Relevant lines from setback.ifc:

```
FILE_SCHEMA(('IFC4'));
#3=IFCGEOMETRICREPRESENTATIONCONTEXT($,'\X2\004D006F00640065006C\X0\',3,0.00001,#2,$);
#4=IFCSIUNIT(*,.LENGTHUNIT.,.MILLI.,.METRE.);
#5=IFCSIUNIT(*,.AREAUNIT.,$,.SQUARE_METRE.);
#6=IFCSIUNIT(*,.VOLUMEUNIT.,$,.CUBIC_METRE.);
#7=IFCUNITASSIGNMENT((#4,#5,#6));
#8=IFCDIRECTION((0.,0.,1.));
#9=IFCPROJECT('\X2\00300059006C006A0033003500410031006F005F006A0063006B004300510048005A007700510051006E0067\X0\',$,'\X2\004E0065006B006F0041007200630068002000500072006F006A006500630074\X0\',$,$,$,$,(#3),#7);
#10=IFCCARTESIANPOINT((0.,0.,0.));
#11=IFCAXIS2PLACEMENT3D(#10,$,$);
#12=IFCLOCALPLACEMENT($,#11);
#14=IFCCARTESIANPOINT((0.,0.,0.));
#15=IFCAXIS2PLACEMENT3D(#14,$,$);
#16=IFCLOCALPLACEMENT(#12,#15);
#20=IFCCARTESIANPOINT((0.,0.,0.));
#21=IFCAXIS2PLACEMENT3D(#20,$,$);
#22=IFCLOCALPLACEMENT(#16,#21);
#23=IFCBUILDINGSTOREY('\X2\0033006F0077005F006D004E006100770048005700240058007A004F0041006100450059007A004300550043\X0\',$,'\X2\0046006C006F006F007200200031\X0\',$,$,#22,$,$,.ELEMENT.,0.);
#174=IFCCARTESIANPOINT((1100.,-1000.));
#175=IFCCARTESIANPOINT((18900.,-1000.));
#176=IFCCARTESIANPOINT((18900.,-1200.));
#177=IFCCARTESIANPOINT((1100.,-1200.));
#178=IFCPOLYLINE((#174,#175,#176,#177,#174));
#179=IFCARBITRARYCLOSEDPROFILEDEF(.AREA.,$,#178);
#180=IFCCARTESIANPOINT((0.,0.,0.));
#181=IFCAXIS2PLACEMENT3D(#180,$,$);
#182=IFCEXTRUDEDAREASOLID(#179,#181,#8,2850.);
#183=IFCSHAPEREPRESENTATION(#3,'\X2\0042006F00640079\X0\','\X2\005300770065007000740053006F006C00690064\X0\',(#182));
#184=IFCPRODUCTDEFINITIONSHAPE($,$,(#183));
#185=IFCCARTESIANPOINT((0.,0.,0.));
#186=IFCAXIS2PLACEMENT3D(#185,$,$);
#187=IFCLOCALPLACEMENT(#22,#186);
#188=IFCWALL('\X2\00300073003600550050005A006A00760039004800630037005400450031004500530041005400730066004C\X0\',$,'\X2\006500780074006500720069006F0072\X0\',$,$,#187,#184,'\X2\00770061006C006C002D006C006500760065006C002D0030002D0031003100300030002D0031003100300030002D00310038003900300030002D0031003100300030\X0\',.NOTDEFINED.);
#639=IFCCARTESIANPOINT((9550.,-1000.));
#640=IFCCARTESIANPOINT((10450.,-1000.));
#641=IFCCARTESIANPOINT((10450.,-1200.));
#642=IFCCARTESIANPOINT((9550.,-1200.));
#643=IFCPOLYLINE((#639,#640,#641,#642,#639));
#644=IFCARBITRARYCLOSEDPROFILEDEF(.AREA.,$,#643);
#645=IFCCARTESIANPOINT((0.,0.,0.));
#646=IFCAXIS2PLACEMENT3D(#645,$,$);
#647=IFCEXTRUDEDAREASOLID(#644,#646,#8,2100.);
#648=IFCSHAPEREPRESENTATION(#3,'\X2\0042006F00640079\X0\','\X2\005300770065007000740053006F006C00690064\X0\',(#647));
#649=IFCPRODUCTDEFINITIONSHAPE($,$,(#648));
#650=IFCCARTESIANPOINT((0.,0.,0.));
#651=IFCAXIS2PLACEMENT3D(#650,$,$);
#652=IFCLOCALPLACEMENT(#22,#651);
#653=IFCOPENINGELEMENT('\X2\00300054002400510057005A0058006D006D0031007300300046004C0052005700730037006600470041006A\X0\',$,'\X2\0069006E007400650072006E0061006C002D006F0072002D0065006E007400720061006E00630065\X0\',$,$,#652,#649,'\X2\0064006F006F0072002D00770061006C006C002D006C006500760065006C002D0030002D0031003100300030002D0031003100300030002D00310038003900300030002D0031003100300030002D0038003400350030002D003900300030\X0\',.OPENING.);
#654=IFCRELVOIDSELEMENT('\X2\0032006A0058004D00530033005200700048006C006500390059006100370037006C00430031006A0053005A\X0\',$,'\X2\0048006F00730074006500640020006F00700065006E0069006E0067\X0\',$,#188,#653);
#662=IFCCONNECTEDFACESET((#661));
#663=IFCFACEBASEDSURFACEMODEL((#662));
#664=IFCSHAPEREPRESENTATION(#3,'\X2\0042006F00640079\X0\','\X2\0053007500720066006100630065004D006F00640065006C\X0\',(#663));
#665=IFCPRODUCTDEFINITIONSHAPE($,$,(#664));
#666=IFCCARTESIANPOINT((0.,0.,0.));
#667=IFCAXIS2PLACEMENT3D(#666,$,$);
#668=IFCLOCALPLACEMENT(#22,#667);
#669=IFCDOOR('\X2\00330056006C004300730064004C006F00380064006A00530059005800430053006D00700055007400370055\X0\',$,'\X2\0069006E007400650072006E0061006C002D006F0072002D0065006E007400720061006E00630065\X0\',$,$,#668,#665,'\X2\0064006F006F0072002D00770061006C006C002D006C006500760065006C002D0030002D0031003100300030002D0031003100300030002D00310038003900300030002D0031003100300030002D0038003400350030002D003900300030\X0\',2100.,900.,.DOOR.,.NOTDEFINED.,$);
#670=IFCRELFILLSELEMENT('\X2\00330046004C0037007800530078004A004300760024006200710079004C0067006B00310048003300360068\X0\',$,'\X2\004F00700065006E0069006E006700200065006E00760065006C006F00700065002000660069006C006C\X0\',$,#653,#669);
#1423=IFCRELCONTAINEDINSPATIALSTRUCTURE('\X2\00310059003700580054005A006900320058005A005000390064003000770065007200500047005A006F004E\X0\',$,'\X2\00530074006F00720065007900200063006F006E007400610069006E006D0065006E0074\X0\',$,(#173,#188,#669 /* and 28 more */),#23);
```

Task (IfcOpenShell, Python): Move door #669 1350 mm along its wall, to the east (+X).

```python
import ifcopenshell
import ifcopenshell.api.geometry
import ifcopenshell.util.placement
import ifcopenshell.util.unit

model = ifcopenshell.open("setback.ifc")
unit_scale = ifcopenshell.util.unit.calculate_unit_scale(model)

door = model.by_id(669)
opening = door.FillsVoids[0].RelatingOpeningElement
wall = opening.VoidsElements[0].RelatingBuildingElement

wall_matrix = ifcopenshell.util.placement.get_local_placement(wall.ObjectPlacement)
shift = wall_matrix[:3, 0] * 1.35 / unit_scale
before = ifcopenshell.util.placement.get_local_placement(door.ObjectPlacement)[:3, 3].copy()

# The door is not placed relative to its opening, so move both.
for product in (opening, door):
    matrix = ifcopenshell.util.placement.get_local_placement(product.ObjectPlacement)
    matrix[:3, 3] += shift
    ifcopenshell.api.geometry.edit_object_placement(model, product=product, matrix=matrix, is_si=False)

after = ifcopenshell.util.placement.get_local_placement(door.ObjectPlacement)[:3, 3]
print("door moved by", (after - before).round(3) + 0.0)

model.write("setback_v2.ifc")
```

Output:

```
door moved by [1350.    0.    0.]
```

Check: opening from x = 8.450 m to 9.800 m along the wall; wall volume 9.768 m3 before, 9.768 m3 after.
